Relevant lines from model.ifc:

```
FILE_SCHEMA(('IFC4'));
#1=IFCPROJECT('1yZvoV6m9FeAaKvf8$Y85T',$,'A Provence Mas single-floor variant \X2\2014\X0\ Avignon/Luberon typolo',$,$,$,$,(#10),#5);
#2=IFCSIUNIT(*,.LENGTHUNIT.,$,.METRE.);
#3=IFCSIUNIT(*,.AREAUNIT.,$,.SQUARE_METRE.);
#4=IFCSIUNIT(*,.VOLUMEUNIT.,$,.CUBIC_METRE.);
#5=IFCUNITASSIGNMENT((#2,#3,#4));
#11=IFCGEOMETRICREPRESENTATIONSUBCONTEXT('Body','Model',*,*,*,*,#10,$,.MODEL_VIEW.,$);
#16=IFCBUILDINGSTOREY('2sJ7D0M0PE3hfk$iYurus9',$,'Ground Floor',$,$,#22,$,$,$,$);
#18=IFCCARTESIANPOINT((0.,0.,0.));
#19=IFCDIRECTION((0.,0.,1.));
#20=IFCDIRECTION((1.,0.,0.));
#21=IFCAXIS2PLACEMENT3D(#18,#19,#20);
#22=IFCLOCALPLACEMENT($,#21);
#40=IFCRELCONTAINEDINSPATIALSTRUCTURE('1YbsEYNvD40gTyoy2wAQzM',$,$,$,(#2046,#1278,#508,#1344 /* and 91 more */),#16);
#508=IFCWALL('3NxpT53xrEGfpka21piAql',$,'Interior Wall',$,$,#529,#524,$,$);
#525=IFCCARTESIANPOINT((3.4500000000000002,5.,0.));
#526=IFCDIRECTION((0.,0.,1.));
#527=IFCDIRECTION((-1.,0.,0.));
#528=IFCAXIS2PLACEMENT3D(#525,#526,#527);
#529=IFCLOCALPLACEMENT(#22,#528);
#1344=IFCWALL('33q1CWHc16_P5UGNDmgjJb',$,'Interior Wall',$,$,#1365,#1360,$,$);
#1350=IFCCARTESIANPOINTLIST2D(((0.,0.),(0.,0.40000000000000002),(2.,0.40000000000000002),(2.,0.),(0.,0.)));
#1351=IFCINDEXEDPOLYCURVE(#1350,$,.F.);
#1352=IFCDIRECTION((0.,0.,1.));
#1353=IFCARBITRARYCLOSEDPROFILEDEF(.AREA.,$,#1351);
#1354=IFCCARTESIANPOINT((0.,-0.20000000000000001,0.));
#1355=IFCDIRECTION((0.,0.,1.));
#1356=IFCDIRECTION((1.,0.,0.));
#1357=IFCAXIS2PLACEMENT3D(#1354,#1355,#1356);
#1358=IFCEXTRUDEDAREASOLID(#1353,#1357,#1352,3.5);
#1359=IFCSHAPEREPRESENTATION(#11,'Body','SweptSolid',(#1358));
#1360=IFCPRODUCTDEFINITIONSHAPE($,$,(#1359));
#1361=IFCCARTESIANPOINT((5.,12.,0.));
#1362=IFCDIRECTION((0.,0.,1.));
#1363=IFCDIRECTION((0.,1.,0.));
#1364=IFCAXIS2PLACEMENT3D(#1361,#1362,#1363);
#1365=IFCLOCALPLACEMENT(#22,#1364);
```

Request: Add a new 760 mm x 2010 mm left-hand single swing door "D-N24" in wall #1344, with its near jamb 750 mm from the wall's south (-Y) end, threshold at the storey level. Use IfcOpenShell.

```python
import numpy as np
import ifcopenshell
import ifcopenshell.api.feature
import ifcopenshell.api.geometry
import ifcopenshell.api.root
import ifcopenshell.api.spatial
import ifcopenshell.geom
import ifcopenshell.util.element
import ifcopenshell.util.placement
import ifcopenshell.util.representation
import ifcopenshell.util.shape
import ifcopenshell.util.unit

model = ifcopenshell.open("model.ifc")
unit_scale = ifcopenshell.util.unit.calculate_unit_scale(model)
settings = ifcopenshell.geom.settings()


def volume(element):
    """Net volume in cubic metres, openings subtracted."""
    shape = ifcopenshell.geom.create_shape(settings, element)
    return ifcopenshell.util.shape.get_volume(shape.geometry)


wall = model.by_guid("33q1CWHc16_P5UGNDmgjJb")
storey = ifcopenshell.util.element.get_container(wall, ifc_class="IfcBuildingStorey")
context = ifcopenshell.util.representation.get_context(model, "Model", "Body", "MODEL_VIEW")
before = volume(wall)

width, height, from_end, sill = 0.76, 2.01, 0.75, 0.0  # metres

# The wall runs along its own X axis, and the end named is its -X end.
wall_shape = ifcopenshell.geom.create_shape(settings, wall)
x, y, z = ifcopenshell.util.shape.get_vertices(wall_shape.geometry).T
start = x.min() + from_end
face, thickness = float(y.min()), float(y.max() - y.min())
wall_matrix = ifcopenshell.util.placement.get_local_placement(wall.ObjectPlacement)
level = ifcopenshell.util.placement.get_local_placement(storey.ObjectPlacement)[2, 3]


def in_wall(x, y):
    """Placement at x, y metres in the wall's axes, at sill height."""
    matrix = wall_matrix.copy()
    matrix[:, 3] = wall_matrix @ np.array([x / unit_scale, y / unit_scale, 0.0, 1.0])
    matrix[2, 3] = level + sill / unit_scale
    return matrix


# Opening: a box that overshoots both wall faces by 50 mm.
opening = ifcopenshell.api.root.create_entity(model, ifc_class="IfcOpeningElement", predefined_type="OPENING")
box = ifcopenshell.api.geometry.add_wall_representation(
    model, context=context, length=width, height=height, thickness=thickness + 0.1
)
ifcopenshell.api.geometry.assign_representation(model, product=opening, representation=box)
ifcopenshell.api.geometry.edit_object_placement(model, product=opening, matrix=in_wall(start, face - 0.05), is_si=False)
ifcopenshell.api.feature.add_feature(model, feature=opening, element=wall)

door = ifcopenshell.api.root.create_entity(model, ifc_class="IfcDoor", name="D-N24", predefined_type="DOOR")
door.OverallWidth, door.OverallHeight = width / unit_scale, height / unit_scale
door.OperationType = "SINGLE_SWING_LEFT"
body = ifcopenshell.api.geometry.add_door_representation(
    model,
    context=context,
    overall_width=door.OverallWidth,
    overall_height=door.OverallHeight,
    operation_type="SINGLE_SWING_LEFT",
    lining_properties={"LiningDepth": thickness / unit_scale, "ThresholdDepth": thickness / unit_scale},
)
ifcopenshell.api.geometry.assign_representation(model, product=door, representation=body)
ifcopenshell.api.spatial.assign_container(model, products=[door], relating_structure=storey)
ifcopenshell.api.feature.add_filling(model, opening=opening, element=door)

# The lining spans the wall, so the door starts at the wall face.
ifcopenshell.api.geometry.edit_object_placement(model, product=door, matrix=in_wall(start, face), is_si=False)

after = volume(wall)

print(f"wall volume {before:.3f} -> {after:.3f} m3")

model.write("model_rev.ifc")
```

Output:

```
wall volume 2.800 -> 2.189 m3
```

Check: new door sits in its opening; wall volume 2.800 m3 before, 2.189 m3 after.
